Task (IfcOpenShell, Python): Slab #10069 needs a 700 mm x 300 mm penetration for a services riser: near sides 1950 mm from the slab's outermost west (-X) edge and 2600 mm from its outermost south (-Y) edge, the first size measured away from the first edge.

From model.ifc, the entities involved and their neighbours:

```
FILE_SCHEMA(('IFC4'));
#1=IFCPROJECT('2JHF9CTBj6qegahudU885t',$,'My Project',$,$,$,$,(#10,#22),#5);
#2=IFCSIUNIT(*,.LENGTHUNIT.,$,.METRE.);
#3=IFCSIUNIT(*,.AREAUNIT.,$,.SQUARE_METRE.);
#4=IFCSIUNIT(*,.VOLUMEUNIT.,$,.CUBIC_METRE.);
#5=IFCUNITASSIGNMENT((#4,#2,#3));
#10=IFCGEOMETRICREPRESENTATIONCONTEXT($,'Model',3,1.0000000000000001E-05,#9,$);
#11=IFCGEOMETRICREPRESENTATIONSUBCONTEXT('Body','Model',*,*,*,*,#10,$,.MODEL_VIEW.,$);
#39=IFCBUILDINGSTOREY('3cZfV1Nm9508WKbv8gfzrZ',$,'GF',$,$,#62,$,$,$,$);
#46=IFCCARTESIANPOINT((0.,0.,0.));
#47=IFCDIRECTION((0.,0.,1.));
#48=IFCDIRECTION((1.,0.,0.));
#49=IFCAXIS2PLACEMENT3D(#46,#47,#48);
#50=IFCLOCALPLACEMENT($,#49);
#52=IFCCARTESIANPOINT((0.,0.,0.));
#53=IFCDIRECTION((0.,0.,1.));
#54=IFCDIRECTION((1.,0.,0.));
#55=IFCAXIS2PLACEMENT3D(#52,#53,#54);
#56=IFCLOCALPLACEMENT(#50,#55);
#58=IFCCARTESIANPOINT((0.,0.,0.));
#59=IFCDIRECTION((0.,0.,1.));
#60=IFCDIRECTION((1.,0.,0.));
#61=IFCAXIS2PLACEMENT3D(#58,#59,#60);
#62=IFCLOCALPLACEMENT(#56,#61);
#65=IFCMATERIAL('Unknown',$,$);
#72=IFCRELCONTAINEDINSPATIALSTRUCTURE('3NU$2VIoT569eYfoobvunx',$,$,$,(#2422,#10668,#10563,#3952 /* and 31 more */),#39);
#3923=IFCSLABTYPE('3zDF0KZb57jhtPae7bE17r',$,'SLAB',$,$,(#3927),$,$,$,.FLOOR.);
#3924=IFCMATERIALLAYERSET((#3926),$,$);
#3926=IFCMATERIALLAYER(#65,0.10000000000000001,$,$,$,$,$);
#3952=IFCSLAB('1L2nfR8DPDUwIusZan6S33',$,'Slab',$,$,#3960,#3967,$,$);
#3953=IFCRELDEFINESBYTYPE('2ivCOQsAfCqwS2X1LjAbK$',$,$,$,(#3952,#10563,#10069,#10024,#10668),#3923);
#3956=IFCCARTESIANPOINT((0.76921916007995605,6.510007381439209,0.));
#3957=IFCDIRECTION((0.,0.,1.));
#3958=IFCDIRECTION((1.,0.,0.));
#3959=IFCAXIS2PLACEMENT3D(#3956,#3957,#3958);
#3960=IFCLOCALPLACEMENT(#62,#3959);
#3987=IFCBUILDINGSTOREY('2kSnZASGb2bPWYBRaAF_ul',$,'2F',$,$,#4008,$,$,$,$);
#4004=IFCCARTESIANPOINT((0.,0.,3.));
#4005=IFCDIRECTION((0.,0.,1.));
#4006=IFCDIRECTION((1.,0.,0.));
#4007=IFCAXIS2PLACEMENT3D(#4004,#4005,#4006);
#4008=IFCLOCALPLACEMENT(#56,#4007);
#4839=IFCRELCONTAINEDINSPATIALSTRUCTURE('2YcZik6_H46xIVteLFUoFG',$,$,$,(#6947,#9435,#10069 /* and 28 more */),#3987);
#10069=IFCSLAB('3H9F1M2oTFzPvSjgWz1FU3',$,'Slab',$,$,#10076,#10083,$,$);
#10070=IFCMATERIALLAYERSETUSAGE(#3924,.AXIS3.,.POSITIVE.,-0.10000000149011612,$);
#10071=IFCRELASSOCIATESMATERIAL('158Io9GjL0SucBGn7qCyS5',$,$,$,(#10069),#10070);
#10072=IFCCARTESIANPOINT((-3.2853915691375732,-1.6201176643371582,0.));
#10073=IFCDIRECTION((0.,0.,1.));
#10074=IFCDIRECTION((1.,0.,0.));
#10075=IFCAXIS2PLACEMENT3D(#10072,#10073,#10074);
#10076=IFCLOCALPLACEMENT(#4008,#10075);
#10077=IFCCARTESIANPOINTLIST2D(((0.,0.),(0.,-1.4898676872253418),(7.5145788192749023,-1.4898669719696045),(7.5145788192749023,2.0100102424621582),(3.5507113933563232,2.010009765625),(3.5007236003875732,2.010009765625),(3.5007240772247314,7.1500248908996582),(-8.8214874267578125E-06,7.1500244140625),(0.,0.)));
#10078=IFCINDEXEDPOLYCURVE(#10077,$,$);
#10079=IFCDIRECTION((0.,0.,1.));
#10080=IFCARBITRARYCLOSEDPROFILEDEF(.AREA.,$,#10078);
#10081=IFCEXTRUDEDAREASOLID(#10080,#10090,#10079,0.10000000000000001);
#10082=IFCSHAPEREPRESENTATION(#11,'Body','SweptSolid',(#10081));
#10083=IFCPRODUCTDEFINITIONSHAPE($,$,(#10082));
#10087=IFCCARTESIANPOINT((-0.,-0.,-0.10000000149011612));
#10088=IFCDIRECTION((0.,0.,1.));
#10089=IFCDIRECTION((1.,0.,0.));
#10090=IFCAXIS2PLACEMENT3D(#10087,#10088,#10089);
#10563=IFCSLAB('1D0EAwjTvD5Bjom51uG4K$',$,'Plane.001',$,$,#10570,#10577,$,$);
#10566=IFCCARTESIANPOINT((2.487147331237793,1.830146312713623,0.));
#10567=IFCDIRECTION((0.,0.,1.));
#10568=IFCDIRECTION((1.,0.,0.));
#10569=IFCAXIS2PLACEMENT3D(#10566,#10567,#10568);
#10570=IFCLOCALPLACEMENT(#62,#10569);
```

```python
import numpy as np
import ifcopenshell
import ifcopenshell.api.feature
import ifcopenshell.api.geometry
import ifcopenshell.api.root
import ifcopenshell.geom
import ifcopenshell.util.placement
import ifcopenshell.util.representation
import ifcopenshell.util.shape
import ifcopenshell.util.unit

model = ifcopenshell.open("model.ifc")
unit_scale = ifcopenshell.util.unit.calculate_unit_scale(model)
settings = ifcopenshell.geom.settings()


def volume(element):
    """Net volume in cubic metres, openings subtracted."""
    shape = ifcopenshell.geom.create_shape(settings, element)
    return ifcopenshell.util.shape.get_volume(shape.geometry)


slab = model.by_id(10069)
before = volume(slab)

# Extent in the slab's own axes, in metres. The edges named are its -X and -Y sides.
slab_shape = ifcopenshell.geom.create_shape(settings, slab)
vertices = ifcopenshell.util.shape.get_vertices(slab_shape.geometry)
x_min, y_min, bottom = vertices.min(axis=0)
top = vertices[:, 2].max()

opening = ifcopenshell.api.root.create_entity(model, ifc_class="IfcOpeningElement", name="Services riser opening", predefined_type="OPENING")
context = ifcopenshell.util.representation.get_context(model, "Model", "Body", "MODEL_VIEW")
width, depth = 0.7, 0.3
outline = [(0.0, 0.0), (width, 0.0), (width, depth), (0.0, depth), (0.0, 0.0)]
# Overshoot both faces by 50 mm so the cut is clean.
shape = ifcopenshell.api.geometry.add_slab_representation(
    model, context=context, depth=top - bottom + 0.1, polyline=outline
)
ifcopenshell.api.geometry.assign_representation(model, product=opening, representation=shape)

matrix = ifcopenshell.util.placement.get_local_placement(slab.ObjectPlacement)
matrix[:, 3] = matrix @ np.append(np.array([x_min + 1.95, y_min + 2.6, bottom - 0.05]) / unit_scale, 1.0)
ifcopenshell.api.geometry.edit_object_placement(model, product=opening, matrix=matrix, is_si=False)
ifcopenshell.api.feature.add_feature(model, feature=opening, element=slab)

after = volume(slab)

print(f"slab volume {before:.3f} -> {after:.3f} m3")

model.write("model_edited.ifc")
```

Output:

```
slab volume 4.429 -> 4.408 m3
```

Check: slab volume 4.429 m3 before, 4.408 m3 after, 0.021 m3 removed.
